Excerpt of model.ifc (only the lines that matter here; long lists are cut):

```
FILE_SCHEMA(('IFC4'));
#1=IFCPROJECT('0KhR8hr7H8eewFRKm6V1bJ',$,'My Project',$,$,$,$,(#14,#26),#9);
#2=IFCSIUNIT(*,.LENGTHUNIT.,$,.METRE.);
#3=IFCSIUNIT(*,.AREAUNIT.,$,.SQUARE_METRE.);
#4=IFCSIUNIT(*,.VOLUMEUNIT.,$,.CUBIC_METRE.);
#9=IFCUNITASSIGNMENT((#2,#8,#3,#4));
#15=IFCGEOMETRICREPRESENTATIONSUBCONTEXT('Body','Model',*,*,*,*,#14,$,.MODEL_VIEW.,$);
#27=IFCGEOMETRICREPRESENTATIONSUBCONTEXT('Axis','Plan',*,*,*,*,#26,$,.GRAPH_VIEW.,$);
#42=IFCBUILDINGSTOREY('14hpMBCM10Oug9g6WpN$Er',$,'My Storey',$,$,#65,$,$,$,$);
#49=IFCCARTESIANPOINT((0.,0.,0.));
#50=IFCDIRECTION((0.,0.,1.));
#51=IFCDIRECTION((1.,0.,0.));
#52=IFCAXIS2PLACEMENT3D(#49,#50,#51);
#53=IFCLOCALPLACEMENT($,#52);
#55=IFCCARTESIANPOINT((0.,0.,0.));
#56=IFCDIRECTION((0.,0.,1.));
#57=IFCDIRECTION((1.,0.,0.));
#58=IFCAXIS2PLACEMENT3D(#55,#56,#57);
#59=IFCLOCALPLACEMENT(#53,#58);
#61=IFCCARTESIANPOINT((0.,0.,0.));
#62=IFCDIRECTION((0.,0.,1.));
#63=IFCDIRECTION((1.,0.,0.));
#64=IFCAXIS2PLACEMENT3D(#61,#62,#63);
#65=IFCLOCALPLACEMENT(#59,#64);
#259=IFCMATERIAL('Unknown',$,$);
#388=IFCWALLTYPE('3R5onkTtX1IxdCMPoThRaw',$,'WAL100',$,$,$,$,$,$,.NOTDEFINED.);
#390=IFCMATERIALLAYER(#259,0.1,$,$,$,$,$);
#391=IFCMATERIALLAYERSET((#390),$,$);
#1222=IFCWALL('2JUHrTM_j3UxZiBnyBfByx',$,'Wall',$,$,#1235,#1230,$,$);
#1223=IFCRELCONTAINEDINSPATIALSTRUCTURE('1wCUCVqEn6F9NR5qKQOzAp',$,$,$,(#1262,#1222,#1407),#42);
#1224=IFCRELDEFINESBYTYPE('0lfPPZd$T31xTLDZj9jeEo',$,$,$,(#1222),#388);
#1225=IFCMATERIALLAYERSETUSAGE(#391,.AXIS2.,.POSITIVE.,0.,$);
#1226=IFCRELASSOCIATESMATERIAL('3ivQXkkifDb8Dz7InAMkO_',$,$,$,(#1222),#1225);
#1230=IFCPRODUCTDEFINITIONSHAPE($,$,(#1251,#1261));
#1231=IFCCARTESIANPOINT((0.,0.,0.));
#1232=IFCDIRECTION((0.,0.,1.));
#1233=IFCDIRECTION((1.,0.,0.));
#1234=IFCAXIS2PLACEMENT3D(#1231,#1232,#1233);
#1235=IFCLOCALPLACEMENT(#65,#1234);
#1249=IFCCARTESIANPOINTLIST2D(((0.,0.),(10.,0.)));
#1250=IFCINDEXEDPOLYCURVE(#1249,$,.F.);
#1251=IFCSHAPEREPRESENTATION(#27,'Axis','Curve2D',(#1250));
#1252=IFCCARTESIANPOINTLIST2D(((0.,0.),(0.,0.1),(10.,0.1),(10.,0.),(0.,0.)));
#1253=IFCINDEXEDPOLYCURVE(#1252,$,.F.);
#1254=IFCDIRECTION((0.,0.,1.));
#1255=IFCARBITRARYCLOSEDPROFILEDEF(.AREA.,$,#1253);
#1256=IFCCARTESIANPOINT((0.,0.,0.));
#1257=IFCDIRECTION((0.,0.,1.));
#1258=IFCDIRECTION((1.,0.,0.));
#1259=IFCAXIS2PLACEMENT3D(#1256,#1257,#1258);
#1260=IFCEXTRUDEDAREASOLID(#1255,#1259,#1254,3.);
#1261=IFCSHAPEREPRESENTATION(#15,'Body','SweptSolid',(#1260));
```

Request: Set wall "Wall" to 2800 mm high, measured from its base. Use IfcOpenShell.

```python
import ifcopenshell
import ifcopenshell.geom
import ifcopenshell.util.representation
import ifcopenshell.util.shape
import ifcopenshell.util.unit

model = ifcopenshell.open("model.ifc")
unit_scale = ifcopenshell.util.unit.calculate_unit_scale(model)
settings = ifcopenshell.geom.settings()


def volume(element):
    """Net volume in cubic metres, openings subtracted."""
    shape = ifcopenshell.geom.create_shape(settings, element)
    return ifcopenshell.util.shape.get_volume(shape.geometry)


wall = model.by_guid("2JUHrTM_j3UxZiBnyBfByx")
before = volume(wall)

body = ifcopenshell.util.representation.get_representation(wall, "Model", "Body")
solid = body.Items[0]
old_height = solid.Depth
solid.Depth = 2.8 / unit_scale
after = volume(wall)

print(f"height {old_height:g} -> {solid.Depth:g}, volume {before:.3f} -> {after:.3f} m3")

model.write("model_v2.ifc")
```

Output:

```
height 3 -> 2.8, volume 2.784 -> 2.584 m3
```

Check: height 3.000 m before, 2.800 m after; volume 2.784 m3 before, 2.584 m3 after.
